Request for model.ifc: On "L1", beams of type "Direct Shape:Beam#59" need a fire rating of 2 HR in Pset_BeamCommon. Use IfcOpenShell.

First a look at what the model holds.

```python
import ifcopenshell
import ifcopenshell.util.element

model = ifcopenshell.open("model.ifc")
print(model.schema)
storey = next(s for s in model.by_type("IfcBuildingStorey") if s.Name == "L1")
beams = [e for e in ifcopenshell.util.element.get_decomposition(storey) if e.is_a("IfcBeam")]
seen = {}
for e in beams:
    element_type = ifcopenshell.util.element.get_type(e)
    key = (element_type.Name if element_type != e and element_type else None, ifcopenshell.util.element.get_pset(e, "Pset_BeamCommon", "FireRating"))
    seen[key] = seen.get(key, 0) + 1
for (name, value), count in sorted(seen.items(), key=str):
    print(count, "x", name, "|", value)
```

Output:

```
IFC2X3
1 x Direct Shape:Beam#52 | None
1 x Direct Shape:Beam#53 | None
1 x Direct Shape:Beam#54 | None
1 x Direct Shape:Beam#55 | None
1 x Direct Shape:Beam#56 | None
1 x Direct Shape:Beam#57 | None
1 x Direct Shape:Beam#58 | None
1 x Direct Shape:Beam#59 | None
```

```python
import ifcopenshell
import ifcopenshell.api.pset
import ifcopenshell.util.element

model = ifcopenshell.open("model.ifc")

storey = next(s for s in model.by_type("IfcBuildingStorey") if s.Name == "L1")
beams = [e for e in ifcopenshell.util.element.get_decomposition(storey) if e.is_a("IfcBeam")]

count = 0
for e in beams:
    element_type = ifcopenshell.util.element.get_type(e)
    if element_type in (None, e) or element_type.Name != "Direct Shape:Beam#59":
        continue
    # add_pset returns the element's existing set when there is one.
    pset = ifcopenshell.api.pset.add_pset(model, product=e, name="Pset_BeamCommon")
    ifcopenshell.api.pset.edit_pset(model, pset=pset, properties={"FireRating": "2 HR"})
    count += 1

print(count, "beams updated")

model.write("model_rev.ifc")
```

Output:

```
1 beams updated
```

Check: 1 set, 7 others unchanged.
